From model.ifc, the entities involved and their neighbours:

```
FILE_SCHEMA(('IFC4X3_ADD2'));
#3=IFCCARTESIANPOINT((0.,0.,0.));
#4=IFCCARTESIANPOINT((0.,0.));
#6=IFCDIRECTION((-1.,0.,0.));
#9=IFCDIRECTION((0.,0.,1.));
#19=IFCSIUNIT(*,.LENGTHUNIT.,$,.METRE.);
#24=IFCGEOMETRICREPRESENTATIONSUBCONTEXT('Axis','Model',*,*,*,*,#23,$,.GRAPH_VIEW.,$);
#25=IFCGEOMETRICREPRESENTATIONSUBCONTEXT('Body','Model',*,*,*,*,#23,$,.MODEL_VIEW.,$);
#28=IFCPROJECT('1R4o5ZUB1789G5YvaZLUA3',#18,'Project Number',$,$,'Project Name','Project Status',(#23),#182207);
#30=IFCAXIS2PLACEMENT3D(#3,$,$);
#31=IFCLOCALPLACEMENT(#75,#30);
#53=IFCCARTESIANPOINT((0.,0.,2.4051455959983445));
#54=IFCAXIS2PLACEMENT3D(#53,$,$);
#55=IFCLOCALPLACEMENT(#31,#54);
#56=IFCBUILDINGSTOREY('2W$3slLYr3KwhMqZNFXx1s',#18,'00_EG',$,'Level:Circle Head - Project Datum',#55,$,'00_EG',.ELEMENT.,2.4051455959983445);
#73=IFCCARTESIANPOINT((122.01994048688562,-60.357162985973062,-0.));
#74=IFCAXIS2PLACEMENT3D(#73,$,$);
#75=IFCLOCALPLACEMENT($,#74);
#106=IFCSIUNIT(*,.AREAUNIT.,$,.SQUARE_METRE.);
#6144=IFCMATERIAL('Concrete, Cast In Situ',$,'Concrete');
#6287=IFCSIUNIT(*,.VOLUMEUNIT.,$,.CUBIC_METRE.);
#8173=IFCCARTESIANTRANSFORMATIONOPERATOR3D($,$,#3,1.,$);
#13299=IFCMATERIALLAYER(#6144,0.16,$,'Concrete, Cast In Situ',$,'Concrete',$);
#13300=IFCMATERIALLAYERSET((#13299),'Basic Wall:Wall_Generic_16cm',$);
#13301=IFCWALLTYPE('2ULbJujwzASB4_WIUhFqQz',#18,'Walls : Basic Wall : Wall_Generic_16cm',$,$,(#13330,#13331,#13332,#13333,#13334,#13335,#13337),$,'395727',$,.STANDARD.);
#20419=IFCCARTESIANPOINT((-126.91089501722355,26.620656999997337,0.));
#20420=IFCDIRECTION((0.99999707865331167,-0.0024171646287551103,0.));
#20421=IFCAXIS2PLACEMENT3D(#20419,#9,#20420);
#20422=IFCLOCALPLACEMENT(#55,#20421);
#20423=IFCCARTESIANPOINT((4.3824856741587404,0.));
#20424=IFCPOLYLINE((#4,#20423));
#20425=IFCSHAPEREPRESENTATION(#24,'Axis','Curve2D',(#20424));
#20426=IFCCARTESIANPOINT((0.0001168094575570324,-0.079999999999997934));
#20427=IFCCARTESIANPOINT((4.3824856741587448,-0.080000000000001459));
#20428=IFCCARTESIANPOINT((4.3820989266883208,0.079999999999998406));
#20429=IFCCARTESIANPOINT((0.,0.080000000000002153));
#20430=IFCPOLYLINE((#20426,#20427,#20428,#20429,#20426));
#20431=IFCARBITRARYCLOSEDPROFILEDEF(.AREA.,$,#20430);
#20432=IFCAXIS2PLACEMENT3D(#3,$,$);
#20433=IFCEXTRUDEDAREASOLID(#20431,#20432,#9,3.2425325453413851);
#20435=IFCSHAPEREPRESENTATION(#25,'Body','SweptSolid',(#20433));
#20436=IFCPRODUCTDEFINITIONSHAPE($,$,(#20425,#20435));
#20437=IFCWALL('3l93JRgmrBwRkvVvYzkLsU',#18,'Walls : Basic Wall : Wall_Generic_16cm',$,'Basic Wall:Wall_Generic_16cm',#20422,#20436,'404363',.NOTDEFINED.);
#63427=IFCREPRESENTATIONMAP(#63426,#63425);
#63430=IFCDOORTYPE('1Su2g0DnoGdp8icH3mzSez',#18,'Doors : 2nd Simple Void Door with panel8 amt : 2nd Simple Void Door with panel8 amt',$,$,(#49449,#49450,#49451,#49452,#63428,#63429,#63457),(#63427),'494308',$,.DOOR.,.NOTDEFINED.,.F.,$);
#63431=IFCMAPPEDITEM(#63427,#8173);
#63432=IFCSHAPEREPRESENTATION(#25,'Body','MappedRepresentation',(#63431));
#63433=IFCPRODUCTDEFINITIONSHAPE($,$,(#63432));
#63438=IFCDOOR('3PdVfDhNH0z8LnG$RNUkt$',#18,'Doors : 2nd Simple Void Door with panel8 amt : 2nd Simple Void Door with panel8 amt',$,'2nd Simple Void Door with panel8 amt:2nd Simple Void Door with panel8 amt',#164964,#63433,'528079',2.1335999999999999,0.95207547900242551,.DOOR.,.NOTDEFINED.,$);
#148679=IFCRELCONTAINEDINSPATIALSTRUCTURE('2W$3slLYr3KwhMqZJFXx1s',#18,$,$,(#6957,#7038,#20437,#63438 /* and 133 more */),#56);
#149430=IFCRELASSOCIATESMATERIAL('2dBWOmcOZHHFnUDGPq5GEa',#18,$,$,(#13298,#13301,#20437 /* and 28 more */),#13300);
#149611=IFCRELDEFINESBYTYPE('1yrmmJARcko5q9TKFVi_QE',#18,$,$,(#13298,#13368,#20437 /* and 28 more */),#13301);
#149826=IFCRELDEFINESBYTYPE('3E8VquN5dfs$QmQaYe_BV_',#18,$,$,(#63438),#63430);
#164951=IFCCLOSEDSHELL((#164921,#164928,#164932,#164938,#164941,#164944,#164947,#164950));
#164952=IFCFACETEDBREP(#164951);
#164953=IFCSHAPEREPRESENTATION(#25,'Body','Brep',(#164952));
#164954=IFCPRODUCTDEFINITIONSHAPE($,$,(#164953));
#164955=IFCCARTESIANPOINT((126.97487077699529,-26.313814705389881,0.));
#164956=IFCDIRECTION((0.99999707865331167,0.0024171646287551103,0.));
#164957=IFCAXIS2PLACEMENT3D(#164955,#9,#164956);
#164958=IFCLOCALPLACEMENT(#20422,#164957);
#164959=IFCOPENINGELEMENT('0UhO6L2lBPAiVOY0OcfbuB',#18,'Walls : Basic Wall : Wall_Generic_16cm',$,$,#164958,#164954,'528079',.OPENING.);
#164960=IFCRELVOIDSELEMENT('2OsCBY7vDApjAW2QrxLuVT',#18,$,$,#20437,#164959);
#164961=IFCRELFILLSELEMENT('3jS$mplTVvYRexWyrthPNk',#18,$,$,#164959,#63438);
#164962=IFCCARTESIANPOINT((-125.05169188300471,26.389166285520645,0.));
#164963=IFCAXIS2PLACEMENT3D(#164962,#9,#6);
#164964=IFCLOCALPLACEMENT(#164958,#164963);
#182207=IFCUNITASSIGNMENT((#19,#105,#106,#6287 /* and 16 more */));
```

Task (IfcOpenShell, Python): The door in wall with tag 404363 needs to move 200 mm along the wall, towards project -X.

```python
import ifcopenshell
import ifcopenshell.api.geometry
import ifcopenshell.util.placement
import ifcopenshell.util.unit

model = ifcopenshell.open("model.ifc")
unit_scale = ifcopenshell.util.unit.calculate_unit_scale(model)

door = model.by_guid("3PdVfDhNH0z8LnG$RNUkt$")
opening = door.FillsVoids[0].RelatingOpeningElement
wall = opening.VoidsElements[0].RelatingBuildingElement

wall_matrix = ifcopenshell.util.placement.get_local_placement(wall.ObjectPlacement)
shift = wall_matrix[:3, 0] * -0.2 / unit_scale
before = ifcopenshell.util.placement.get_local_placement(door.ObjectPlacement)[:3, 3].copy()

# The door is placed relative to its opening, so it follows when the opening moves.
matrix = ifcopenshell.util.placement.get_local_placement(opening.ObjectPlacement)
matrix[:3, 3] += shift
ifcopenshell.api.geometry.edit_object_placement(
    model, product=opening, matrix=matrix, is_si=False, should_transform_children=True
)

after = ifcopenshell.util.placement.get_local_placement(door.ObjectPlacement)[:3, 3]
print("door moved by", (after - before).round(3) + 0.0)

model.write("model_edited.ifc")
```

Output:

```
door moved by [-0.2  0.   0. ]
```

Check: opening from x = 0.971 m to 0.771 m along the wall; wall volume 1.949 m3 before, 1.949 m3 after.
